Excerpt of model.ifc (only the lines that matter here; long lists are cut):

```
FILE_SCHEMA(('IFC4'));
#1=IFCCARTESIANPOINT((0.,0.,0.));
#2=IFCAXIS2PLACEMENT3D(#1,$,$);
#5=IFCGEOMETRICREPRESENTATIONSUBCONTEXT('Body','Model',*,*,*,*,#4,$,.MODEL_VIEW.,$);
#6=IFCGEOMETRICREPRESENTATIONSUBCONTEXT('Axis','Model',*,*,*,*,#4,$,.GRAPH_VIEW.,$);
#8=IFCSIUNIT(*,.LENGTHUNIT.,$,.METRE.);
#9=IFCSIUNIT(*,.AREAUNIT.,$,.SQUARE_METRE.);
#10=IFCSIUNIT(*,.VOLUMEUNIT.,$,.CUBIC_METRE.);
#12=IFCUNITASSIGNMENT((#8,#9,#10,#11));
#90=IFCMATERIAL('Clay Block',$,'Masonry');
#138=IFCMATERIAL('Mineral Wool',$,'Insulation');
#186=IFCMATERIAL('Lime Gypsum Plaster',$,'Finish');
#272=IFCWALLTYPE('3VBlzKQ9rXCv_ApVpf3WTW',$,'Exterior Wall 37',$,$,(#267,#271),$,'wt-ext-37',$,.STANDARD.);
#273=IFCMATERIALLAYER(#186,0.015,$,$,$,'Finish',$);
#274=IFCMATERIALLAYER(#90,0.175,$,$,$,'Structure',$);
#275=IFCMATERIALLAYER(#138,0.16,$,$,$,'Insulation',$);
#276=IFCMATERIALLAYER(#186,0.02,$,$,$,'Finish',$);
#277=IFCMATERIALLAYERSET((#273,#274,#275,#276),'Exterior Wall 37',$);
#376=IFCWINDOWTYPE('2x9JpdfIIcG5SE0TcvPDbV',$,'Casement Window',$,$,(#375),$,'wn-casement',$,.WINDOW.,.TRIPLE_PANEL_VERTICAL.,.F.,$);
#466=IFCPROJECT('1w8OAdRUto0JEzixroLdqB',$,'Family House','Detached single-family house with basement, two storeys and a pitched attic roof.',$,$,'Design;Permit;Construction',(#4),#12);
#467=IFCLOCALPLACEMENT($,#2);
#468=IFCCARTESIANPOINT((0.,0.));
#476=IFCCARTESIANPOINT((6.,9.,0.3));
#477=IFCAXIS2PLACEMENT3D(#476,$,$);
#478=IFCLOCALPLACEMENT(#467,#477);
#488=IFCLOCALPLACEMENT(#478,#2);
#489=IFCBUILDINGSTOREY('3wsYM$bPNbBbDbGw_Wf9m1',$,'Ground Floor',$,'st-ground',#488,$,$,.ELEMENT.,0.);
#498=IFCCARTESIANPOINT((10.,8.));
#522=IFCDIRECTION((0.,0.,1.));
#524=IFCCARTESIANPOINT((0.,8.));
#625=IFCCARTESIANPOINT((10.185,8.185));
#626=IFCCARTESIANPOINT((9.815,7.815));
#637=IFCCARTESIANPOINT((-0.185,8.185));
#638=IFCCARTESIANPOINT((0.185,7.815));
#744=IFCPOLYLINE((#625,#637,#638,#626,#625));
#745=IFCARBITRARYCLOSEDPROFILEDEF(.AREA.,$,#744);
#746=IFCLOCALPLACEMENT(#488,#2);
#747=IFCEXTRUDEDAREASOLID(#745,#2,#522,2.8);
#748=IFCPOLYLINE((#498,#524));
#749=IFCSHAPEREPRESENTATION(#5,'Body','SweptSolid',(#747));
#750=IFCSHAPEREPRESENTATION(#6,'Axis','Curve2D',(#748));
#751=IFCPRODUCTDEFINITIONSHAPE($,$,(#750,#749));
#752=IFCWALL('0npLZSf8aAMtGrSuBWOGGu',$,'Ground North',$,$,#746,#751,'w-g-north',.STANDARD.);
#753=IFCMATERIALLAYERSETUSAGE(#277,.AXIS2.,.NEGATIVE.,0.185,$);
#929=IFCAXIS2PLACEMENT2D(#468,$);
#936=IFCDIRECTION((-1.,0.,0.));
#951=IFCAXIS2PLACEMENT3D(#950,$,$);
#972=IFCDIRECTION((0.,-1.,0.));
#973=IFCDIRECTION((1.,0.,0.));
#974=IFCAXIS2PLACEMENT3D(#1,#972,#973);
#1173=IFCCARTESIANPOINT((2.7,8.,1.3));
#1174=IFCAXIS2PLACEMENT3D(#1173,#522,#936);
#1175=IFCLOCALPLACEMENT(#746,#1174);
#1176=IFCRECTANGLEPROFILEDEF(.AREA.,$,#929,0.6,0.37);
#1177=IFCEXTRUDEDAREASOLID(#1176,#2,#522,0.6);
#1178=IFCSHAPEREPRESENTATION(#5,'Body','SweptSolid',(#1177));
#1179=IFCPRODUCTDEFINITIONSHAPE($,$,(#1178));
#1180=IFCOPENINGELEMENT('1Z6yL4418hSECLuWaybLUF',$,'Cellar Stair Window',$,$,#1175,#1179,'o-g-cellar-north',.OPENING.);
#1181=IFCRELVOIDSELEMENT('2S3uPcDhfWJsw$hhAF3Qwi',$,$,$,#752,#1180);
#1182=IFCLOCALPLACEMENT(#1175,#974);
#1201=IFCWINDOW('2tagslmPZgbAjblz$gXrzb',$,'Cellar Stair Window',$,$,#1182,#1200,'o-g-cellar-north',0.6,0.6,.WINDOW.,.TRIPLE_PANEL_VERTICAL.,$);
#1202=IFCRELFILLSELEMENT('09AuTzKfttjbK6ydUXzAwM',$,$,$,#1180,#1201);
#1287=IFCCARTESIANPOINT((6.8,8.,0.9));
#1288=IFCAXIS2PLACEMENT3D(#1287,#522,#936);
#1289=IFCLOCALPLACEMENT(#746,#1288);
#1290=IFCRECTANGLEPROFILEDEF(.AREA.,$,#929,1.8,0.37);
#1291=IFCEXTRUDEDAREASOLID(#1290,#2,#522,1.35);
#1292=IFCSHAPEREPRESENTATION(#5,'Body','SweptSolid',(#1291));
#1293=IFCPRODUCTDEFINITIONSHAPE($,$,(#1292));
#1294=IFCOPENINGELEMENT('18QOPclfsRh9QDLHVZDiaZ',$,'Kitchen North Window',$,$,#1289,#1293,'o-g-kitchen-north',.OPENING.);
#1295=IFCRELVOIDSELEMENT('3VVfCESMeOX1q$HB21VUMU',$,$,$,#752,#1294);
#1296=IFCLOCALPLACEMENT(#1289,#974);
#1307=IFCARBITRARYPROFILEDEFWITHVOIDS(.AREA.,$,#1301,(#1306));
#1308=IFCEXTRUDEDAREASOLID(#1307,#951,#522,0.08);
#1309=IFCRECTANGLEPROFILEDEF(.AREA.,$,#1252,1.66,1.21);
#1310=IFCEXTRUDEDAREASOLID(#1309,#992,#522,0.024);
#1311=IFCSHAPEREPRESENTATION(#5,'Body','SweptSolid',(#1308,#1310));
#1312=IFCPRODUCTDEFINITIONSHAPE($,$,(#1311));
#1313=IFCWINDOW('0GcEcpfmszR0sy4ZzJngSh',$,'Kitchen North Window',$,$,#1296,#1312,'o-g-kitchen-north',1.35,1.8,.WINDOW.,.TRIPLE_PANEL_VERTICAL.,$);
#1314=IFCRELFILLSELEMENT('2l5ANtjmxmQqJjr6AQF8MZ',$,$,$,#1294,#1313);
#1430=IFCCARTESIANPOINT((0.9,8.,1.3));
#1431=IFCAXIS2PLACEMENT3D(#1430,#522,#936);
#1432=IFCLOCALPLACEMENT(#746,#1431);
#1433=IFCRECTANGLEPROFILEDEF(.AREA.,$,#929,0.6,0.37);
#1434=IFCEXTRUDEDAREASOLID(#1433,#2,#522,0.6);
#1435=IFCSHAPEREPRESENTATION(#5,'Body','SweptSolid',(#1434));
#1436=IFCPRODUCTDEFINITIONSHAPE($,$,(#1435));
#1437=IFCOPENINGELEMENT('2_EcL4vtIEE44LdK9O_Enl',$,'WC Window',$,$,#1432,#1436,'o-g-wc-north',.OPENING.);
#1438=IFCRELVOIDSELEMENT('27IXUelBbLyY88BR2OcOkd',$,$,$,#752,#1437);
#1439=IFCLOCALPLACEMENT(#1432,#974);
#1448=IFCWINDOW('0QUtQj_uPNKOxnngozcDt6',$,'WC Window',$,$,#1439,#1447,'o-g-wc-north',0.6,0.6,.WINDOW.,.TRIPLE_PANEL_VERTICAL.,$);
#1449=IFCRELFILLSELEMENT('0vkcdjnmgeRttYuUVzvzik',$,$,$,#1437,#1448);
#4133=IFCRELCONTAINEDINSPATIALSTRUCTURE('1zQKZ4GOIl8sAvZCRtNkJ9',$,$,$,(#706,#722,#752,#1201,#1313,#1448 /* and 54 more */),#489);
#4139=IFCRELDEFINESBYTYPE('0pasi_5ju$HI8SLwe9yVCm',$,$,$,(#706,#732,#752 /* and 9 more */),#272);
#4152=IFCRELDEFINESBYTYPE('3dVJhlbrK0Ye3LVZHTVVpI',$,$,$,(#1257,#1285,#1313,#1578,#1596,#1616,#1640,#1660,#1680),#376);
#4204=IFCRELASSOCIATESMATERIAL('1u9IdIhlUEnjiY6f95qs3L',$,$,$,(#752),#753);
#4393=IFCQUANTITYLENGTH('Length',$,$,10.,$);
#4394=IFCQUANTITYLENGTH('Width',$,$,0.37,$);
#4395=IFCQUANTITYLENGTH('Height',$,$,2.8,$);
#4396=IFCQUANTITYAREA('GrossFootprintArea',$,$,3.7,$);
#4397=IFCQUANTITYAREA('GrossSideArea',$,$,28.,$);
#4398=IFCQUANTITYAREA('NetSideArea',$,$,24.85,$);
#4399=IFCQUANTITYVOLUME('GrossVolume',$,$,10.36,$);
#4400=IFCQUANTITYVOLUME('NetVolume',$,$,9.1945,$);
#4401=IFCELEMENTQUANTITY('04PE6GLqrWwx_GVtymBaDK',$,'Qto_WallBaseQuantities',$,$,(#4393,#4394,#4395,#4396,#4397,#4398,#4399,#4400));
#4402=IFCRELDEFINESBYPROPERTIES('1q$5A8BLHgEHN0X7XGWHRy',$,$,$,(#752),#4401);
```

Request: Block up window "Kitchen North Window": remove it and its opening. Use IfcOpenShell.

```python
import ifcopenshell
import ifcopenshell.api.feature
import ifcopenshell.api.pset
import ifcopenshell.api.root
import ifcopenshell.geom
import ifcopenshell.util.element
import ifcopenshell.util.shape
import ifcopenshell.util.unit

model = ifcopenshell.open("model.ifc")
area_scale = ifcopenshell.util.unit.calculate_unit_scale(model, "AREAUNIT")
volume_scale = ifcopenshell.util.unit.calculate_unit_scale(model, "VOLUMEUNIT")
settings = ifcopenshell.geom.settings()


def volume(element):
    """Net volume in cubic metres, openings subtracted."""
    shape = ifcopenshell.geom.create_shape(settings, element)
    return ifcopenshell.util.shape.get_volume(shape.geometry)


window = model.by_guid("0GcEcpfmszR0sy4ZzJngSh")
opening = window.FillsVoids[0].RelatingOpeningElement
wall = opening.VoidsElements[0].RelatingBuildingElement
before = volume(wall)

ifcopenshell.api.root.remove_product(model, product=window)
ifcopenshell.api.feature.remove_feature(model, feature=opening)

after = volume(wall)
thickness = 0.37  # wall thickness in metres

# Update the wall's stored quantities.
qto = model.by_id(ifcopenshell.util.element.get_pset(wall, "Qto_WallBaseQuantities", should_inherit=False)["id"])
ifcopenshell.api.pset.edit_qto(model, qto=qto, properties={
    "NetSideArea": after / thickness / area_scale,
    "NetVolume": after / volume_scale,
})

print(f"wall volume {before:.3f} -> {after:.3f} m3")

model.write("model_rev.ifc")
```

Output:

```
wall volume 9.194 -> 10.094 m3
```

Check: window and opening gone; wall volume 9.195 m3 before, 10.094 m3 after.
